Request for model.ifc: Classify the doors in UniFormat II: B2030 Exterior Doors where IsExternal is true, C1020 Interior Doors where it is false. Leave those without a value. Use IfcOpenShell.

First a look at what the model holds.

```python
import ifcopenshell
import ifcopenshell.util.element

model = ifcopenshell.open("model.ifc")
print(model.schema)
print("classifications:", [c.Name for c in model.by_type("IfcClassification")])
values = [ifcopenshell.util.element.get_pset(e, "Pset_DoorCommon", "IsExternal") for e in model.by_type("IfcDoor")]
for value in (True, False, None):
    print("IsExternal", value, values.count(value))
```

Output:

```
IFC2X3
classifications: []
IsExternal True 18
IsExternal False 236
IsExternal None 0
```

```python
import ifcopenshell
import ifcopenshell.api.classification
import ifcopenshell.util.element

model = ifcopenshell.open("model.ifc")

# IFC2X3 requires Source and Edition and has no link from the project to the system.
system = model.create_entity("IfcClassification", Source="ASTM", Edition="E1557", Name="UniFormat II")

doors = model.by_type("IfcDoor")
external = {e: ifcopenshell.util.element.get_pset(e, "Pset_DoorCommon", "IsExternal") for e in doors}
for flag, code, name in ((True, "B2030", "Exterior Doors"), (False, "C1020", "Interior Doors")):
    products = [e for e in doors if external[e] is flag]
    ifcopenshell.api.classification.add_reference(
        model, products=products, classification=system, identification=code, name=name
    )
    print(code, len(products))

model.write("model_edited.ifc")
```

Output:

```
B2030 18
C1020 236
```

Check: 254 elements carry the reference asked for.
